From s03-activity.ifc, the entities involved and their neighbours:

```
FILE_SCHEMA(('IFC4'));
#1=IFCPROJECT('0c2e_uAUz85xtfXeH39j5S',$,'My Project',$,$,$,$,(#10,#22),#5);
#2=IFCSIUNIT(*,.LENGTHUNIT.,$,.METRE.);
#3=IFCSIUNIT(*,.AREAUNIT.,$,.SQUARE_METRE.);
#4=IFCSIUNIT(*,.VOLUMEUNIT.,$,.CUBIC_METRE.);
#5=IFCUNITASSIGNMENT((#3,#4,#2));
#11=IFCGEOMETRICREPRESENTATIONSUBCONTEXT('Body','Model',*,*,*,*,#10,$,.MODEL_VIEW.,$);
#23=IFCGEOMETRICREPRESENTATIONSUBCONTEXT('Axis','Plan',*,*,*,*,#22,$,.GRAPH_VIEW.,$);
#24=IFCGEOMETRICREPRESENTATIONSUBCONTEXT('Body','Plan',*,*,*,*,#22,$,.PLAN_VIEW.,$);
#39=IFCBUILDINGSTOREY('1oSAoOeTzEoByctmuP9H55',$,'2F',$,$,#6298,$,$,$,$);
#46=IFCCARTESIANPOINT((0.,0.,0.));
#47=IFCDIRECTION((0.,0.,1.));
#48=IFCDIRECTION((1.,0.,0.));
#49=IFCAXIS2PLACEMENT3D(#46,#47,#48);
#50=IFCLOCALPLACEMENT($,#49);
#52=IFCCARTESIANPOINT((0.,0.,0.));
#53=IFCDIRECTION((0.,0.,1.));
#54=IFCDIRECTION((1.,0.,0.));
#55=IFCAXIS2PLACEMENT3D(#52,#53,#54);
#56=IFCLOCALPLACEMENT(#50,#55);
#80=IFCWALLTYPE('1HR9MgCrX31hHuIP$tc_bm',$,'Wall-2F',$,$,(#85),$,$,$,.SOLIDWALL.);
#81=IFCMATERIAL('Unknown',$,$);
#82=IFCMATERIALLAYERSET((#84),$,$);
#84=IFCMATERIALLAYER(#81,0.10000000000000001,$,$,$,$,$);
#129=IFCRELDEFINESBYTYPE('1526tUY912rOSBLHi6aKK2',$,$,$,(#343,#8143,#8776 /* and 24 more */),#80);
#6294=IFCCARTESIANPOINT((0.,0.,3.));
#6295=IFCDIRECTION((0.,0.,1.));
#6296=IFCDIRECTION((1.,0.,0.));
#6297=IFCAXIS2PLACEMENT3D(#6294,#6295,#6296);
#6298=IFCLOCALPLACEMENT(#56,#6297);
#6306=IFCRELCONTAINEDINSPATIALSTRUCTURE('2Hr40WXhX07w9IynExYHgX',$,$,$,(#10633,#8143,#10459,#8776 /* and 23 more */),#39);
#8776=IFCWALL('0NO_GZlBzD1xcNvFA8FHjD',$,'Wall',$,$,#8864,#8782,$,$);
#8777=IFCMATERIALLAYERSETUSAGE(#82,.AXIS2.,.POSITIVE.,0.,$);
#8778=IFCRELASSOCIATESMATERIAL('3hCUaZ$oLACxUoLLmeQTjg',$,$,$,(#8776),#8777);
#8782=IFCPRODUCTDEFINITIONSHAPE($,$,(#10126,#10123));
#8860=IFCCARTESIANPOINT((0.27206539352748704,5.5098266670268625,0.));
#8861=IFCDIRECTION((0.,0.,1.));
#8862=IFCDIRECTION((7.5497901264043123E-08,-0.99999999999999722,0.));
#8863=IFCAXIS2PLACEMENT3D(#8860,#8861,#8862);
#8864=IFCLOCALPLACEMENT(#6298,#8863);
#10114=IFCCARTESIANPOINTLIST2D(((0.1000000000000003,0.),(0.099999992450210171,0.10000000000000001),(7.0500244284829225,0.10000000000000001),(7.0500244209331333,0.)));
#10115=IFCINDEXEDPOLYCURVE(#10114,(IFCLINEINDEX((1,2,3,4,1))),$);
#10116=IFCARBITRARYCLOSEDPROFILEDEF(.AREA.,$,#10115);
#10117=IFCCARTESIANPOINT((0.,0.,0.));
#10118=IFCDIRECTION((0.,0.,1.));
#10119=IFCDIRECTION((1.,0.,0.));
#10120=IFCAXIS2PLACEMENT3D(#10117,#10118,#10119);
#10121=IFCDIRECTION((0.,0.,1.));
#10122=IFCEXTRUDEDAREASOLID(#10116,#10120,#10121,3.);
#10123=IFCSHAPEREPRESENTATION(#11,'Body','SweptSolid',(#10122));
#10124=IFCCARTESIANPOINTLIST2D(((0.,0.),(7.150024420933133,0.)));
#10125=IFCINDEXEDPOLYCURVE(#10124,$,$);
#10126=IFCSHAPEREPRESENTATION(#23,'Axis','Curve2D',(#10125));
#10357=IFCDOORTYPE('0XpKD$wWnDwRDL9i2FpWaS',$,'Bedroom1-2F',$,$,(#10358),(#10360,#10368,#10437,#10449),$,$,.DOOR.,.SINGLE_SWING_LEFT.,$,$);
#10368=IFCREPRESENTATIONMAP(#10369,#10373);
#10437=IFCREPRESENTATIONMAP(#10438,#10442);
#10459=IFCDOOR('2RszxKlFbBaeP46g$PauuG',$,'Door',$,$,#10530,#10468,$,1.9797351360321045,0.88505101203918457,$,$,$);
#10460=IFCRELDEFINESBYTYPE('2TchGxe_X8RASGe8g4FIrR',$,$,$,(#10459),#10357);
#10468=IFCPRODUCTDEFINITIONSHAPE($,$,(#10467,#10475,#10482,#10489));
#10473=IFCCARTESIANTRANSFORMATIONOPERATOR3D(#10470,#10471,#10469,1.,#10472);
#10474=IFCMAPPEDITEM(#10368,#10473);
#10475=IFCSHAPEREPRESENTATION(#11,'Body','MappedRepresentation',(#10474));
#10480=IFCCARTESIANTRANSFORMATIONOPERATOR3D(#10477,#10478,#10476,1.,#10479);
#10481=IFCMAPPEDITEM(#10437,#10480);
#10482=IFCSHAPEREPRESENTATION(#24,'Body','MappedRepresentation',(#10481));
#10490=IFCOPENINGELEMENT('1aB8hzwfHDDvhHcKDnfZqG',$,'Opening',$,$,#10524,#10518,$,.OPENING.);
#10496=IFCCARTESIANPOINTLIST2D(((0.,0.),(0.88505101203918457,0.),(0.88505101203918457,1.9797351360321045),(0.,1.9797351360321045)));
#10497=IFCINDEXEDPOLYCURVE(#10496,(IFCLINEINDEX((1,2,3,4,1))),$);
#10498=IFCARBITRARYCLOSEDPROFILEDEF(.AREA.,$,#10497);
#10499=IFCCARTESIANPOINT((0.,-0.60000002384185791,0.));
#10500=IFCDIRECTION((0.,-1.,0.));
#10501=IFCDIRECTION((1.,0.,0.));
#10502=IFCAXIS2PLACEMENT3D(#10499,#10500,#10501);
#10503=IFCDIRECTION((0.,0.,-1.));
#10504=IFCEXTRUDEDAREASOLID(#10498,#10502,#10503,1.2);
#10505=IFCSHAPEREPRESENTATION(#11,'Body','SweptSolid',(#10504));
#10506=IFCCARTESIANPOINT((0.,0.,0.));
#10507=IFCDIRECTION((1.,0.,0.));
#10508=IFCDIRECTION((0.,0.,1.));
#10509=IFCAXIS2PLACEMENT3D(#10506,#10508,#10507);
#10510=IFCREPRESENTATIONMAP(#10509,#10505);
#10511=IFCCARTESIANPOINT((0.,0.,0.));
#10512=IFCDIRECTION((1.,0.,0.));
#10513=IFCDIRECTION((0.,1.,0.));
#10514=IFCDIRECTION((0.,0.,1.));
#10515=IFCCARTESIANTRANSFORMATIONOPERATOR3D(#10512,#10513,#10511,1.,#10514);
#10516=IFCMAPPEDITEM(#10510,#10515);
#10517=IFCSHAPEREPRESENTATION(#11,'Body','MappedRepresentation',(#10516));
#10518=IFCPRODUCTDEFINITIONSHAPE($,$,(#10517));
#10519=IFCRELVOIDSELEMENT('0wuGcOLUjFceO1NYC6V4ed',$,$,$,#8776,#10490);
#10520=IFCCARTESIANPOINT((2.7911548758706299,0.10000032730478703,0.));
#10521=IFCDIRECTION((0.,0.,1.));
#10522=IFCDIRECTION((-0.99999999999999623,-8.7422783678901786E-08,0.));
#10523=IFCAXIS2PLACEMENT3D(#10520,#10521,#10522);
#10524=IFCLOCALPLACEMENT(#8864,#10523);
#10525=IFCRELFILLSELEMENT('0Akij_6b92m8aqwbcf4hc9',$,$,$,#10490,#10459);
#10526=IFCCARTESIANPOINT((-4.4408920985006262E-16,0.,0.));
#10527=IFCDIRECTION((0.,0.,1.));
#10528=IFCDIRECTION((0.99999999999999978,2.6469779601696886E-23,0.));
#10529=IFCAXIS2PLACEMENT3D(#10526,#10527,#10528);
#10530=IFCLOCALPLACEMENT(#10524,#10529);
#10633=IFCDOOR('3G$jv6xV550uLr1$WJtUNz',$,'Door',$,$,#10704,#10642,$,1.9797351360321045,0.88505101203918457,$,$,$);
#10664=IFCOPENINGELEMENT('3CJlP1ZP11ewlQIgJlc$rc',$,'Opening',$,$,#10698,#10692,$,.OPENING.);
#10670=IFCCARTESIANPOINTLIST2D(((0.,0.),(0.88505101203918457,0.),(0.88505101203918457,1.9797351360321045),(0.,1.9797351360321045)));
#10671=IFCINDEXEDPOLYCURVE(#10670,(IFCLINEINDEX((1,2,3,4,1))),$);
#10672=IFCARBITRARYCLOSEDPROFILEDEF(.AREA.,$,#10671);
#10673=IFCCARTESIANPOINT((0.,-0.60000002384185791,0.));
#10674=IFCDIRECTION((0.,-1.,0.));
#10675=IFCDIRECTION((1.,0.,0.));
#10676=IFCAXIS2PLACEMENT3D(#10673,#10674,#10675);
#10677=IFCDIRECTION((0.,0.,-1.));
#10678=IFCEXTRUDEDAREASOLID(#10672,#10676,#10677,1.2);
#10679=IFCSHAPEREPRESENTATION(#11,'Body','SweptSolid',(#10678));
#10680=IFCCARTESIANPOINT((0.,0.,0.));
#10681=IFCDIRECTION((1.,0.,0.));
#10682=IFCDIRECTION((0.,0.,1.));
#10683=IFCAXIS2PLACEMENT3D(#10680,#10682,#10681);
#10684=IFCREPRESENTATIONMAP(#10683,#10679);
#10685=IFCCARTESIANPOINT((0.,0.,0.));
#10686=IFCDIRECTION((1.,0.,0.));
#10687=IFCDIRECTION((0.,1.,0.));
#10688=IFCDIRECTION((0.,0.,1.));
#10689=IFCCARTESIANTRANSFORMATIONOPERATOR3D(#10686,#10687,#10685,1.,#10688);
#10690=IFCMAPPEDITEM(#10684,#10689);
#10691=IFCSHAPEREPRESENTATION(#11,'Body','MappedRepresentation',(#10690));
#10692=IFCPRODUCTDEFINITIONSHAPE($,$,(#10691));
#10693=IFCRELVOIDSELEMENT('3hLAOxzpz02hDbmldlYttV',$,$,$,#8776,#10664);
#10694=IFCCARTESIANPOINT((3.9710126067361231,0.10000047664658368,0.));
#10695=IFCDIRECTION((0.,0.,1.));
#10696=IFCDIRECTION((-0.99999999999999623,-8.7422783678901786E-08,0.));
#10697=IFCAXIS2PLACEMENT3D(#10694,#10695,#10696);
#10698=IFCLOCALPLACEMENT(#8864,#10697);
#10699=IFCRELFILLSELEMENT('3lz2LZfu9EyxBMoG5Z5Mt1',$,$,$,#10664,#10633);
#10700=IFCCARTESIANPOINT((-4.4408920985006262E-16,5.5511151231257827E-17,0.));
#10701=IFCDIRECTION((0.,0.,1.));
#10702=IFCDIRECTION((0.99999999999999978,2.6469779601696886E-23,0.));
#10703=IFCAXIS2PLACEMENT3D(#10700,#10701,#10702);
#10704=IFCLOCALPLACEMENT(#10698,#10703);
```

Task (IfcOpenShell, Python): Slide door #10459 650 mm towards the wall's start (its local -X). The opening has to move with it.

```python
import ifcopenshell
import ifcopenshell.api.geometry
import ifcopenshell.util.placement

model = ifcopenshell.open("s03-activity.ifc")

door = model.by_id(10459)
opening = door.FillsVoids[0].RelatingOpeningElement
wall = opening.VoidsElements[0].RelatingBuildingElement

wall_matrix = ifcopenshell.util.placement.get_local_placement(wall.ObjectPlacement)
shift = wall_matrix[:3, 0] * -0.65
before = ifcopenshell.util.placement.get_local_placement(door.ObjectPlacement)[:3, 3].copy()

# The door is placed relative to its opening, so it follows when the opening moves.
matrix = ifcopenshell.util.placement.get_local_placement(opening.ObjectPlacement)
matrix[:3, 3] += shift
ifcopenshell.api.geometry.edit_object_placement(
    model, product=opening, matrix=matrix, is_si=False, should_transform_children=True
)

after = ifcopenshell.util.placement.get_local_placement(door.ObjectPlacement)[:3, 3]
print("door moved by", (after - before).round(3) + 0.0)

model.write("s03-activity_edited.ifc")
```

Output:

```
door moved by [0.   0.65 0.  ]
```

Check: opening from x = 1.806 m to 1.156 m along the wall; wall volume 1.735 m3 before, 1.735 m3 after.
